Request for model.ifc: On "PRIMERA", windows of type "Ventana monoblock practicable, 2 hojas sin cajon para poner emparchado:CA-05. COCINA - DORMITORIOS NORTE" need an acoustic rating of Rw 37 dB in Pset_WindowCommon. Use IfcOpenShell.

First a look at what the model holds.

```python
import ifcopenshell
import ifcopenshell.util.element

model = ifcopenshell.open("model.ifc")
print(model.schema)
storey = next(s for s in model.by_type("IfcBuildingStorey") if s.Name == "PRIMERA")
windows = [e for e in ifcopenshell.util.element.get_decomposition(storey) if e.is_a("IfcWindow")]
seen = {}
for e in windows:
    element_type = ifcopenshell.util.element.get_type(e)
    key = (element_type.Name if element_type != e and element_type else None, ifcopenshell.util.element.get_pset(e, "Pset_WindowCommon", "AcousticRating"))
    seen[key] = seen.get(key, 0) + 1
for (name, value), count in sorted(seen.items(), key=str):
    print(count, "x", name, "|", value)
```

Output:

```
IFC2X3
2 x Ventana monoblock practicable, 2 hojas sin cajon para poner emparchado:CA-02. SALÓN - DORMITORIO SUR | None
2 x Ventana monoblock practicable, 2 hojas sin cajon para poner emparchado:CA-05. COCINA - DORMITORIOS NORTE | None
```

```python
import ifcopenshell
import ifcopenshell.api.pset
import ifcopenshell.util.element

model = ifcopenshell.open("model.ifc")

storey = next(s for s in model.by_type("IfcBuildingStorey") if s.Name == "PRIMERA")
windows = [e for e in ifcopenshell.util.element.get_decomposition(storey) if e.is_a("IfcWindow")]

count = 0
for e in windows:
    element_type = ifcopenshell.util.element.get_type(e)
    if element_type in (None, e) or element_type.Name != "Ventana monoblock practicable, 2 hojas sin cajon para poner emparchado:CA-05. COCINA - DORMITORIOS NORTE":
        continue
    # add_pset returns the element's existing set when there is one.
    pset = ifcopenshell.api.pset.add_pset(model, product=e, name="Pset_WindowCommon")
    ifcopenshell.api.pset.edit_pset(model, pset=pset, properties={"AcousticRating": "Rw 37 dB"})
    count += 1

print(count, "windows updated")

model.write("model_v2.ifc")
```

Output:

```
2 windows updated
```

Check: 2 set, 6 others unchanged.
